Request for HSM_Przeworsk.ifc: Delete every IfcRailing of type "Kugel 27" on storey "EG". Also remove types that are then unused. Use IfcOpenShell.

First a look at what the model holds.

```python
import ifcopenshell
import ifcopenshell.util.element

model = ifcopenshell.open("HSM_Przeworsk.ifc")
print(model.schema)
storey = next(s for s in model.by_type("IfcBuildingStorey") if s.Name == "EG")
railings = [e for e in ifcopenshell.util.element.get_decomposition(storey) if e.is_a("IfcRailing")]
seen = {}
for e in railings:
    element_type = ifcopenshell.util.element.get_type(e)
    name = element_type.Name if element_type not in (None, e) else None
    seen[name] = seen.get(name, 0) + 1
for name, count in sorted(seen.items(), key=str):
    print(count, "x", name)
```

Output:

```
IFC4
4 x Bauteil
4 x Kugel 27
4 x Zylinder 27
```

```python
import ifcopenshell
import ifcopenshell.api.root
import ifcopenshell.util.element

model = ifcopenshell.open("HSM_Przeworsk.ifc")

storey = next(s for s in model.by_type("IfcBuildingStorey") if s.Name == "EG")
railings = [e for e in ifcopenshell.util.element.get_decomposition(storey) if e.is_a("IfcRailing")]
targets = [e for e in railings if (t := ifcopenshell.util.element.get_type(e)) not in (None, e) and t.Name == "Kugel 27"]
types = {ifcopenshell.util.element.get_type(e) for e in targets} - {None, *targets}

for e in targets:
    ifcopenshell.api.root.remove_product(model, product=e)
print(len(targets), "removed")

unused = [t for t in types if not ifcopenshell.util.element.get_types(t)]
for t in unused:
    ifcopenshell.api.root.remove_product(model, product=t)
print(len(unused), "unused types removed")

model.write("HSM_Przeworsk_edited.ifc")
```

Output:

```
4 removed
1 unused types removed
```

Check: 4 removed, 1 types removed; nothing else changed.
